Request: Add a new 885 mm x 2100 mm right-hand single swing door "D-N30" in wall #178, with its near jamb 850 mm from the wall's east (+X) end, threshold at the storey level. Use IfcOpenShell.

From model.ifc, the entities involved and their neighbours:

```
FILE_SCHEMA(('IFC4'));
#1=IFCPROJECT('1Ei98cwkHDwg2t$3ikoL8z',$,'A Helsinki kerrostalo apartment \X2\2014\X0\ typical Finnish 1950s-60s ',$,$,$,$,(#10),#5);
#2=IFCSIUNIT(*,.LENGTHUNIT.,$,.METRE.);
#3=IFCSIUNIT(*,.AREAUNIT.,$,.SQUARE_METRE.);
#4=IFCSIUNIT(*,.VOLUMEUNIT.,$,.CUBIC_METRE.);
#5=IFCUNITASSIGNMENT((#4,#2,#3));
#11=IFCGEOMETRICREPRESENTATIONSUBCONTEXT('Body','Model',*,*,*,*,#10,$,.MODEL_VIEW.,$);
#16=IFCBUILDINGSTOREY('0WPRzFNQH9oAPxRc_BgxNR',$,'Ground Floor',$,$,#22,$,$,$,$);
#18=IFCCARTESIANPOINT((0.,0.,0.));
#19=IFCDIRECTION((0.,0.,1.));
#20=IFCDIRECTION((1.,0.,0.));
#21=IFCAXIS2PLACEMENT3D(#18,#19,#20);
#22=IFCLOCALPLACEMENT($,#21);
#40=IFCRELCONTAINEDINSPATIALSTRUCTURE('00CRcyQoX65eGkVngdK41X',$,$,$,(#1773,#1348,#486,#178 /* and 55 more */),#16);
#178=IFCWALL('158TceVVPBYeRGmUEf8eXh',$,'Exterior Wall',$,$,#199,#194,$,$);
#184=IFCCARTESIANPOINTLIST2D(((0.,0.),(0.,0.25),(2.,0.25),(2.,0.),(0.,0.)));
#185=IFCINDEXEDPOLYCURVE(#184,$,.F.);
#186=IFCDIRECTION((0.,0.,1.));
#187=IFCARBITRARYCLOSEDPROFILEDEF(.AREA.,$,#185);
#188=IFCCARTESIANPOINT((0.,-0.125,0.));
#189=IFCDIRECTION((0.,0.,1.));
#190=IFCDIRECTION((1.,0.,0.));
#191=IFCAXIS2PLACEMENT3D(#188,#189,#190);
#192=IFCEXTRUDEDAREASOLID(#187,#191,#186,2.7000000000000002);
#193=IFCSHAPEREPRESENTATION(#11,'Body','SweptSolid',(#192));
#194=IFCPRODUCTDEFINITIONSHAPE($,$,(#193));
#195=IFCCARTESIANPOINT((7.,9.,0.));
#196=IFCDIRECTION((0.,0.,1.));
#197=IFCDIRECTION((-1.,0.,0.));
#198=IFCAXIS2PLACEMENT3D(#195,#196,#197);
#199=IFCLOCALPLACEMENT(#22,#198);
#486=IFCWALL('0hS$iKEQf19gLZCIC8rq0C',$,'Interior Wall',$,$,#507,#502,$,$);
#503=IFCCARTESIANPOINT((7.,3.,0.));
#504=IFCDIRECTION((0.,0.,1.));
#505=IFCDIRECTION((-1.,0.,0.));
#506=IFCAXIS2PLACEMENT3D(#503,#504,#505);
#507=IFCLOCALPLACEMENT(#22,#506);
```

```python
import numpy as np
import ifcopenshell
import ifcopenshell.api.feature
import ifcopenshell.api.geometry
import ifcopenshell.api.root
import ifcopenshell.api.spatial
import ifcopenshell.geom
import ifcopenshell.util.element
import ifcopenshell.util.placement
import ifcopenshell.util.representation
import ifcopenshell.util.shape
import ifcopenshell.util.unit

model = ifcopenshell.open("model.ifc")
unit_scale = ifcopenshell.util.unit.calculate_unit_scale(model)
settings = ifcopenshell.geom.settings()


def volume(element):
    """Net volume in cubic metres, openings subtracted."""
    shape = ifcopenshell.geom.create_shape(settings, element)
    return ifcopenshell.util.shape.get_volume(shape.geometry)


wall = model.by_guid("158TceVVPBYeRGmUEf8eXh")
storey = ifcopenshell.util.element.get_container(wall, ifc_class="IfcBuildingStorey")
context = ifcopenshell.util.representation.get_context(model, "Model", "Body", "MODEL_VIEW")
before = volume(wall)

width, height, from_end, sill = 0.885, 2.1, 0.85, 0.0  # metres

# The wall runs along its own X axis, and the end named is its -X end.
wall_shape = ifcopenshell.geom.create_shape(settings, wall)
x, y, z = ifcopenshell.util.shape.get_vertices(wall_shape.geometry).T
start = x.min() + from_end
face, thickness = float(y.min()), float(y.max() - y.min())
wall_matrix = ifcopenshell.util.placement.get_local_placement(wall.ObjectPlacement)
level = ifcopenshell.util.placement.get_local_placement(storey.ObjectPlacement)[2, 3]


def in_wall(x, y):
    """Placement at x, y metres in the wall's axes, at sill height."""
    matrix = wall_matrix.copy()
    matrix[:, 3] = wall_matrix @ np.array([x / unit_scale, y / unit_scale, 0.0, 1.0])
    matrix[2, 3] = level + sill / unit_scale
    return matrix


# Opening: a box that overshoots both wall faces by 50 mm.
opening = ifcopenshell.api.root.create_entity(model, ifc_class="IfcOpeningElement", predefined_type="OPENING")
box = ifcopenshell.api.geometry.add_wall_representation(
    model, context=context, length=width, height=height, thickness=thickness + 0.1
)
ifcopenshell.api.geometry.assign_representation(model, product=opening, representation=box)
ifcopenshell.api.geometry.edit_object_placement(model, product=opening, matrix=in_wall(start, face - 0.05), is_si=False)
ifcopenshell.api.feature.add_feature(model, feature=opening, element=wall)

door = ifcopenshell.api.root.create_entity(model, ifc_class="IfcDoor", name="D-N30", predefined_type="DOOR")
door.OverallWidth, door.OverallHeight = width / unit_scale, height / unit_scale
door.OperationType = "SINGLE_SWING_RIGHT"
body = ifcopenshell.api.geometry.add_door_representation(
    model,
    context=context,
    overall_width=door.OverallWidth,
    overall_height=door.OverallHeight,
    operation_type="SINGLE_SWING_RIGHT",
    lining_properties={"LiningDepth": thickness / unit_scale, "ThresholdDepth": thickness / unit_scale},
)
ifcopenshell.api.geometry.assign_representation(model, product=door, representation=body)
ifcopenshell.api.spatial.assign_container(model, products=[door], relating_structure=storey)
ifcopenshell.api.feature.add_filling(model, opening=opening, element=door)

# The lining spans the wall, so the door starts at the wall face.
ifcopenshell.api.geometry.edit_object_placement(model, product=door, matrix=in_wall(start, face), is_si=False)

after = volume(wall)

print(f"wall volume {before:.3f} -> {after:.3f} m3")

model.write("model-out.ifc")
```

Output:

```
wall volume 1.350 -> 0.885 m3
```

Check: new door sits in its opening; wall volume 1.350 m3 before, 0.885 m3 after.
